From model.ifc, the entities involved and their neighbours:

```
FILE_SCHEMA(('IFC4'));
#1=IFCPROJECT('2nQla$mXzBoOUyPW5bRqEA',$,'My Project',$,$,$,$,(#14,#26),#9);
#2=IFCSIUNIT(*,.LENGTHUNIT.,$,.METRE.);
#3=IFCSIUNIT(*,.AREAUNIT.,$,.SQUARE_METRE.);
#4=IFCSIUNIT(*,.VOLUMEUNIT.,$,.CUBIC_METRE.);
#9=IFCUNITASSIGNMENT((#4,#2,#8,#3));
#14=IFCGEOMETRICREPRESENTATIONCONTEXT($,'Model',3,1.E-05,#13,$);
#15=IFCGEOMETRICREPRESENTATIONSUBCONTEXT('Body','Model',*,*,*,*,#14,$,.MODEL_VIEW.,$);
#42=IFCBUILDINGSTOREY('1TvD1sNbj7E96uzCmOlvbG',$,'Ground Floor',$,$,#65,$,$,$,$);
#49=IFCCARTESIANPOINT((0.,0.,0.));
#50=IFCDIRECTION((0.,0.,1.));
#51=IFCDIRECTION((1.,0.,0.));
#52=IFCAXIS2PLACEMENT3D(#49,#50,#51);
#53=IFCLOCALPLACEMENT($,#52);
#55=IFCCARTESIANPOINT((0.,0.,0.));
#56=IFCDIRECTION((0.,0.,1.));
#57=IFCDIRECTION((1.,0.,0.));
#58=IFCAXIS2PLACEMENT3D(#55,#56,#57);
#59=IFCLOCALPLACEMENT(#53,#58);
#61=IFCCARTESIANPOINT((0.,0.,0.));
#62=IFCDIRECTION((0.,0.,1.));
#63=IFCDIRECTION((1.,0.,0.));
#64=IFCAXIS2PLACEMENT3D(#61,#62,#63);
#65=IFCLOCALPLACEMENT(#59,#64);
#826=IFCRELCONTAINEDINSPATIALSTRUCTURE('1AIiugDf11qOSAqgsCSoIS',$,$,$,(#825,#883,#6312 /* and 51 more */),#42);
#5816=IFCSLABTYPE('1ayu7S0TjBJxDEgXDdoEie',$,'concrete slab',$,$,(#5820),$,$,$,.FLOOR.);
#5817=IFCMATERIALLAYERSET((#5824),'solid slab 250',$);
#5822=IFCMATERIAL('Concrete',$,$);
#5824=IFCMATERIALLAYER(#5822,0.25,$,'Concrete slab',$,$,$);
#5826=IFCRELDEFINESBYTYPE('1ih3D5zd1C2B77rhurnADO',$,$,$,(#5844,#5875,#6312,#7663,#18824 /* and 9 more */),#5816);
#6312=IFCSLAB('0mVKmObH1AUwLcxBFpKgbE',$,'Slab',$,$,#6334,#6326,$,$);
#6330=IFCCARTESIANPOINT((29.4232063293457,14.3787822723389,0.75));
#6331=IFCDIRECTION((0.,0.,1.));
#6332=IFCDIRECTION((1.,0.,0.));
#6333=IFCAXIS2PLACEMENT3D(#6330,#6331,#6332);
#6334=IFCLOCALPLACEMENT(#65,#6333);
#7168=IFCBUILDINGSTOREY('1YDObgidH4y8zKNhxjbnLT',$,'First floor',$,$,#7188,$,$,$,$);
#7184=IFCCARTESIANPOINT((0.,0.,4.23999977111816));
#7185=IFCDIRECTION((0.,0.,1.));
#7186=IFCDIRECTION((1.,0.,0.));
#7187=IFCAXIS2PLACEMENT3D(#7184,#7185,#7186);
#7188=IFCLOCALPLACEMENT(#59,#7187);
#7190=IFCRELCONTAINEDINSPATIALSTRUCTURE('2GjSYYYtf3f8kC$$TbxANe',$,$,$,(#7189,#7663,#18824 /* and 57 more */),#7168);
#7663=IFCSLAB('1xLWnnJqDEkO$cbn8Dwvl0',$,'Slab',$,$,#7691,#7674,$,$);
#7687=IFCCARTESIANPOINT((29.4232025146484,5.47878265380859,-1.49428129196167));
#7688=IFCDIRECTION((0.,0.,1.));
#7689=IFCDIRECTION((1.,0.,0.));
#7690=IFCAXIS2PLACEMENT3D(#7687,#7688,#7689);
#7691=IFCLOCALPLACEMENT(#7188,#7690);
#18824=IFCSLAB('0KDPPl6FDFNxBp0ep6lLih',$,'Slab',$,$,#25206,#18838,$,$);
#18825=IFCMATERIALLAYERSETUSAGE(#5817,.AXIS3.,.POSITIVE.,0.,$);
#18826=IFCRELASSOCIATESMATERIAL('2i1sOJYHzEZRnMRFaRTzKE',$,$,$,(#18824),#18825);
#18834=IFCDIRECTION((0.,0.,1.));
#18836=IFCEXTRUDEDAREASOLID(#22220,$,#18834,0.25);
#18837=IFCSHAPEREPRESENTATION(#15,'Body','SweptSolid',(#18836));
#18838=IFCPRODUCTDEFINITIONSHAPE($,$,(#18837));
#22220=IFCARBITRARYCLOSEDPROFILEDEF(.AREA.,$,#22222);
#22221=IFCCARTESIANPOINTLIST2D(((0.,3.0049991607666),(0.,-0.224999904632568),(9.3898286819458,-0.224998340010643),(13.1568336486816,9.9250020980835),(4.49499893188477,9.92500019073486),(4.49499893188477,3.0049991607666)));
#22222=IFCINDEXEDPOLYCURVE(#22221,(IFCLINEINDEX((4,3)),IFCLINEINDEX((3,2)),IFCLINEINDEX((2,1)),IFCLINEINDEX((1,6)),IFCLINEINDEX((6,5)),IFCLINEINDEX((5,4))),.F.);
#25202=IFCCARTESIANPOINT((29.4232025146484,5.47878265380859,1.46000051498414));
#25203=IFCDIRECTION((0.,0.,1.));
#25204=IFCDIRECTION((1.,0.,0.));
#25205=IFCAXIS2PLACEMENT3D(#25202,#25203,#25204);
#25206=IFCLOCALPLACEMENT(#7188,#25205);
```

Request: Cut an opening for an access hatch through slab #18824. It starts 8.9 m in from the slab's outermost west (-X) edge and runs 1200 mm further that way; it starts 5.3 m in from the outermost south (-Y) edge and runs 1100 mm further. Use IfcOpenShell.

```python
import numpy as np
import ifcopenshell
import ifcopenshell.api.feature
import ifcopenshell.api.geometry
import ifcopenshell.api.root
import ifcopenshell.geom
import ifcopenshell.util.placement
import ifcopenshell.util.representation
import ifcopenshell.util.shape
import ifcopenshell.util.unit

model = ifcopenshell.open("model.ifc")
unit_scale = ifcopenshell.util.unit.calculate_unit_scale(model)
settings = ifcopenshell.geom.settings()


def volume(element):
    """Net volume in cubic metres, openings subtracted."""
    shape = ifcopenshell.geom.create_shape(settings, element)
    return ifcopenshell.util.shape.get_volume(shape.geometry)


slab = model.by_guid("0KDPPl6FDFNxBp0ep6lLih")
before = volume(slab)

# Extent in the slab's own axes, in metres. The edges named are its -X and -Y sides.
slab_shape = ifcopenshell.geom.create_shape(settings, slab)
vertices = ifcopenshell.util.shape.get_vertices(slab_shape.geometry)
x_min, y_min, bottom = vertices.min(axis=0)
top = vertices[:, 2].max()

opening = ifcopenshell.api.root.create_entity(model, ifc_class="IfcOpeningElement", name="Access hatch opening", predefined_type="OPENING")
context = ifcopenshell.util.representation.get_context(model, "Model", "Body", "MODEL_VIEW")
width, depth = 1.2, 1.1
outline = [(0.0, 0.0), (width, 0.0), (width, depth), (0.0, depth), (0.0, 0.0)]
# Overshoot both faces by 50 mm so the cut is clean.
shape = ifcopenshell.api.geometry.add_slab_representation(
    model, context=context, depth=top - bottom + 0.1, polyline=outline
)
ifcopenshell.api.geometry.assign_representation(model, product=opening, representation=shape)

matrix = ifcopenshell.util.placement.get_local_placement(slab.ObjectPlacement)
matrix[:, 3] = matrix @ np.append(np.array([x_min + 8.9, y_min + 5.3, bottom - 0.05]) / unit_scale, 1.0)
ifcopenshell.api.geometry.edit_object_placement(model, product=opening, matrix=matrix, is_si=False)
ifcopenshell.api.feature.add_feature(model, feature=opening, element=slab)

after = volume(slab)

print(f"slab volume {before:.3f} -> {after:.3f} m3")

model.write("model_v2.ifc")
```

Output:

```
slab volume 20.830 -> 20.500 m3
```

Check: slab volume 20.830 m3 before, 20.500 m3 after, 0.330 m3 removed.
